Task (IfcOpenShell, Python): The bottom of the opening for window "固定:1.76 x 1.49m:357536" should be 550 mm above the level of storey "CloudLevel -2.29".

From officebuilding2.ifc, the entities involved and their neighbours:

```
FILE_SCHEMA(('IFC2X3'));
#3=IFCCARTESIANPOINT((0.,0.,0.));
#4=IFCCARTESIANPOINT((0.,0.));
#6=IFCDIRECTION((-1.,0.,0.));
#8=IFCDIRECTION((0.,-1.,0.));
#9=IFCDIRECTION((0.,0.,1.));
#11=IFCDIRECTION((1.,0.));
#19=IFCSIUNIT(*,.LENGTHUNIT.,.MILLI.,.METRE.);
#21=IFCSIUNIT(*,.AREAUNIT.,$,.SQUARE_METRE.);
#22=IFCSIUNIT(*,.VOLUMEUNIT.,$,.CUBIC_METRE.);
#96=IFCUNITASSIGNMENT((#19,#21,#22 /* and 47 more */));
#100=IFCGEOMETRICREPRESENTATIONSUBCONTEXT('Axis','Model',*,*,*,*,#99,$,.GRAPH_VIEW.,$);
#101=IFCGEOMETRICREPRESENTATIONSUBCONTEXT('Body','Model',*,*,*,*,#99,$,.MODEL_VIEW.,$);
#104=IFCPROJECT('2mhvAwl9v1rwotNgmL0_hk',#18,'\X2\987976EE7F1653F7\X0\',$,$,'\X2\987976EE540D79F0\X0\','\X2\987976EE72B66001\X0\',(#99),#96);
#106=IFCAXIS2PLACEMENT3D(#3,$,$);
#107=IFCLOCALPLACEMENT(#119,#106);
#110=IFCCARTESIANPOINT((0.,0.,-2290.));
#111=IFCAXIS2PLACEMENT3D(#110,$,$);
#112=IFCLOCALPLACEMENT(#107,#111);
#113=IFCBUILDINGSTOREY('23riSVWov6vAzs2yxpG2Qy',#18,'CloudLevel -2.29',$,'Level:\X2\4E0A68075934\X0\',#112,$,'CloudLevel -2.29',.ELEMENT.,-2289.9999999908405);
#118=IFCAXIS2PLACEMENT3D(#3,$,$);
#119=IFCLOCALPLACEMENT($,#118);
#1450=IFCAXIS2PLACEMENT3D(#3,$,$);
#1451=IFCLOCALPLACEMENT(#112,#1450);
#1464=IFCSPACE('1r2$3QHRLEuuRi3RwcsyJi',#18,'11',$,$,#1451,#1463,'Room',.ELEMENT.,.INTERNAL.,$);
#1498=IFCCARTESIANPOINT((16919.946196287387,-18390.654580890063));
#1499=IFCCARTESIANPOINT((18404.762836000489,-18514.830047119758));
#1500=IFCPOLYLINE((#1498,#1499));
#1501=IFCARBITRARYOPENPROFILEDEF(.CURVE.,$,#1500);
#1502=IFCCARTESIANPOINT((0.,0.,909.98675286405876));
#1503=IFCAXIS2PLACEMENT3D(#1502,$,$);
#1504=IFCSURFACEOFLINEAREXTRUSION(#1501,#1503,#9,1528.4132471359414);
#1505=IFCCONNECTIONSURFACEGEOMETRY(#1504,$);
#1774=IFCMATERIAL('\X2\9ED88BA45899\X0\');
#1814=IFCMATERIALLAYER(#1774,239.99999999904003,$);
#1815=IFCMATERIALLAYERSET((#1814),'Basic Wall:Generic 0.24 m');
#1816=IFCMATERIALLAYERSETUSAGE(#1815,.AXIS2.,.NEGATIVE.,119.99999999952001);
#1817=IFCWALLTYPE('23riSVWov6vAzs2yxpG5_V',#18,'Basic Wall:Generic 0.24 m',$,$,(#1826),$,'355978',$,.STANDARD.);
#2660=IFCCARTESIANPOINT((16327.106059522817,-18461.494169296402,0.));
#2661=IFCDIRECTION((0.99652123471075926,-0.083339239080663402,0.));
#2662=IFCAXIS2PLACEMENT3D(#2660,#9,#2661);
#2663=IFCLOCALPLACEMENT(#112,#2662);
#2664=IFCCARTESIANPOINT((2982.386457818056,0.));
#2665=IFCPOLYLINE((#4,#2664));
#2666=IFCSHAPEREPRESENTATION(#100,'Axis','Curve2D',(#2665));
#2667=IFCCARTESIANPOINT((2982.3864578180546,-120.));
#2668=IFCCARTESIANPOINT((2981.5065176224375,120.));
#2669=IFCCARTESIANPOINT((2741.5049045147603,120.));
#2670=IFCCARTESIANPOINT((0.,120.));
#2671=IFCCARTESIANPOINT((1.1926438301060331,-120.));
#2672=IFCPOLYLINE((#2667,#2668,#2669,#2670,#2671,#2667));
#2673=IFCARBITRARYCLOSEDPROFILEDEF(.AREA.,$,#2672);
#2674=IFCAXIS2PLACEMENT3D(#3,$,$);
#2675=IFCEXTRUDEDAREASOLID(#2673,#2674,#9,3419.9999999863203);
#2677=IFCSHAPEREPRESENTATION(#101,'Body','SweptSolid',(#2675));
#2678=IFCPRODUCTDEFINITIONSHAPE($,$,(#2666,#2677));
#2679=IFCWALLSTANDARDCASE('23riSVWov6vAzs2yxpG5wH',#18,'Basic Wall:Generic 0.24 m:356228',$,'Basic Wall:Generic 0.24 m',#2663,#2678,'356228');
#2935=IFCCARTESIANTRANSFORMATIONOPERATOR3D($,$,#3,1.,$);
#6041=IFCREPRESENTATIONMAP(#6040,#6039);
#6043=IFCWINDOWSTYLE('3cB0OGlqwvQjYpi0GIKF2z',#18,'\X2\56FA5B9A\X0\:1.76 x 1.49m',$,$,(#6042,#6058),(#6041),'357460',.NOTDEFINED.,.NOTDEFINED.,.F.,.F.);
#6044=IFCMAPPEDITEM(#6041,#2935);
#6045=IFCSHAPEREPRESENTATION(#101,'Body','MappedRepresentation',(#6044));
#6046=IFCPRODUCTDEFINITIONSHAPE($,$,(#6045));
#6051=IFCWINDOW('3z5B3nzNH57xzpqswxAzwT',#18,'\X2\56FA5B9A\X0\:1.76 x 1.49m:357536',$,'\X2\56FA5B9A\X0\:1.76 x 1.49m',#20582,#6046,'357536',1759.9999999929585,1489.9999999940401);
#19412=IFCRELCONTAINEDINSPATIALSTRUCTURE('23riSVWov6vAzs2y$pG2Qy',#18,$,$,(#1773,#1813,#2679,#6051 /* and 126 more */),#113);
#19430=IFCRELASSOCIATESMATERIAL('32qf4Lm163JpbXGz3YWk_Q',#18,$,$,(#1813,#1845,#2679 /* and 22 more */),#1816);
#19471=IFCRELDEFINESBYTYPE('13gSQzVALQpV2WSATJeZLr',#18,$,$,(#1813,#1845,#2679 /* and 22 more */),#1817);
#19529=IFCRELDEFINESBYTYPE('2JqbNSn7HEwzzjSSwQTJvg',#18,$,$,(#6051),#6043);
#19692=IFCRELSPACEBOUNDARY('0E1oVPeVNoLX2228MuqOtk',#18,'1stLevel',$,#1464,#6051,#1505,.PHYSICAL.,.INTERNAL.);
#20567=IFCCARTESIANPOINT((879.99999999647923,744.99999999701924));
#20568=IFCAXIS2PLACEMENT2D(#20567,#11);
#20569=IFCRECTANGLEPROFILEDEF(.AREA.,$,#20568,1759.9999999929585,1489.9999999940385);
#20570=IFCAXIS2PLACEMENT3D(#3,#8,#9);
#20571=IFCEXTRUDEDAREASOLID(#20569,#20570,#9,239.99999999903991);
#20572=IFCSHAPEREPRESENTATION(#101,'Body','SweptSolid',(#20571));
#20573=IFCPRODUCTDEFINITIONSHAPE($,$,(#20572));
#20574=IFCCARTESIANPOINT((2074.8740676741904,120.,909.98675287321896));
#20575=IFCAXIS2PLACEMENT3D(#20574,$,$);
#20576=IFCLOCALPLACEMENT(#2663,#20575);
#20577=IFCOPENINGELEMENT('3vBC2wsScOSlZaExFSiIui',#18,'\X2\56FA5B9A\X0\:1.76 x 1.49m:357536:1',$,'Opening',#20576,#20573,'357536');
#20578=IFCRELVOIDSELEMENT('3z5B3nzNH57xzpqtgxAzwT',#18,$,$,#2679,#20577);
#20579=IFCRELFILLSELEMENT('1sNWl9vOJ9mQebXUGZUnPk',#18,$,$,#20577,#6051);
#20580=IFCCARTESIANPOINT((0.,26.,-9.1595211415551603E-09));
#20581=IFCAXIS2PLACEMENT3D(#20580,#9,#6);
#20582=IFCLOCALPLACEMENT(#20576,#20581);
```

```python
import numpy as np
import ifcopenshell
import ifcopenshell.api.geometry
import ifcopenshell.geom
import ifcopenshell.util.element
import ifcopenshell.util.placement
import ifcopenshell.util.shape
import ifcopenshell.util.unit

model = ifcopenshell.open("officebuilding2.ifc")
unit_scale = ifcopenshell.util.unit.calculate_unit_scale(model)

window = model.by_guid("3z5B3nzNH57xzpqswxAzwT")
opening = window.FillsVoids[0].RelatingOpeningElement
storey = ifcopenshell.util.element.get_container(window, ifc_class="IfcBuildingStorey")
level = ifcopenshell.util.placement.get_local_placement(storey.ObjectPlacement)[2, 3]

# The opening's origin need not be at the sill, so measure its lowest point.
shape = ifcopenshell.geom.create_shape(ifcopenshell.geom.settings(), opening)
bottom = ifcopenshell.util.shape.get_shape_bottom_elevation(shape, shape.geometry) / unit_scale
dz = level + 550.0 - bottom

shift = np.array([0.0, 0.0, dz])
# The window is placed relative to its opening, so it follows when the opening moves.
matrix = ifcopenshell.util.placement.get_local_placement(opening.ObjectPlacement)
matrix[:3, 3] += shift
ifcopenshell.api.geometry.edit_object_placement(
    model, product=opening, matrix=matrix, is_si=False, should_transform_children=True
)

# Space boundary surfaces are stored in each space's coordinates; move them too.
for rel in window.ProvidesBoundaries:
    if not rel.ConnectionGeometry:
        continue
    surface = rel.ConnectionGeometry.SurfaceOnRelatingElement
    space_matrix = ifcopenshell.util.placement.get_local_placement(rel.RelatingSpace.ObjectPlacement)
    point = np.array(surface.Position.Location.Coordinates) + space_matrix[:3, :3].T @ shift
    surface.Position = model.createIfcAxis2Placement3D(
        model.createIfcCartesianPoint(point.tolist()), surface.Position.Axis, surface.Position.RefDirection
    )

print(f"moved by {dz * unit_scale:+.3f} m")

model.write("officebuilding2_rev.ifc")
```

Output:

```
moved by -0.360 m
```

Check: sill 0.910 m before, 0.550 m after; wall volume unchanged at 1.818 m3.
